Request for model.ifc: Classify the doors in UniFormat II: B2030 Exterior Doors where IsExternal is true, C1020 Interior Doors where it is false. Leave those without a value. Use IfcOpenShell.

First a look at what the model holds.

```python
import ifcopenshell
import ifcopenshell.util.element

model = ifcopenshell.open("model.ifc")
print(model.schema)
print("classifications:", [c.Name for c in model.by_type("IfcClassification")])
values = [ifcopenshell.util.element.get_pset(e, "Pset_DoorCommon", "IsExternal") for e in model.by_type("IfcDoor")]
for value in (True, False, None):
    print("IsExternal", value, values.count(value))
```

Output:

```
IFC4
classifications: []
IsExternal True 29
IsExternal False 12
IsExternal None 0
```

```python
import ifcopenshell
import ifcopenshell.api.classification
import ifcopenshell.util.element

model = ifcopenshell.open("model.ifc")

system = ifcopenshell.api.classification.add_classification(model, classification="UniFormat II")

doors = model.by_type("IfcDoor")
external = {e: ifcopenshell.util.element.get_pset(e, "Pset_DoorCommon", "IsExternal") for e in doors}
for flag, code, name in ((True, "B2030", "Exterior Doors"), (False, "C1020", "Interior Doors")):
    products = [e for e in doors if external[e] is flag]
    ifcopenshell.api.classification.add_reference(
        model, products=products, classification=system, identification=code, name=name
    )
    print(code, len(products))

model.write("model_updated.ifc")
```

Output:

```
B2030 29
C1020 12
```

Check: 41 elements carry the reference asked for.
